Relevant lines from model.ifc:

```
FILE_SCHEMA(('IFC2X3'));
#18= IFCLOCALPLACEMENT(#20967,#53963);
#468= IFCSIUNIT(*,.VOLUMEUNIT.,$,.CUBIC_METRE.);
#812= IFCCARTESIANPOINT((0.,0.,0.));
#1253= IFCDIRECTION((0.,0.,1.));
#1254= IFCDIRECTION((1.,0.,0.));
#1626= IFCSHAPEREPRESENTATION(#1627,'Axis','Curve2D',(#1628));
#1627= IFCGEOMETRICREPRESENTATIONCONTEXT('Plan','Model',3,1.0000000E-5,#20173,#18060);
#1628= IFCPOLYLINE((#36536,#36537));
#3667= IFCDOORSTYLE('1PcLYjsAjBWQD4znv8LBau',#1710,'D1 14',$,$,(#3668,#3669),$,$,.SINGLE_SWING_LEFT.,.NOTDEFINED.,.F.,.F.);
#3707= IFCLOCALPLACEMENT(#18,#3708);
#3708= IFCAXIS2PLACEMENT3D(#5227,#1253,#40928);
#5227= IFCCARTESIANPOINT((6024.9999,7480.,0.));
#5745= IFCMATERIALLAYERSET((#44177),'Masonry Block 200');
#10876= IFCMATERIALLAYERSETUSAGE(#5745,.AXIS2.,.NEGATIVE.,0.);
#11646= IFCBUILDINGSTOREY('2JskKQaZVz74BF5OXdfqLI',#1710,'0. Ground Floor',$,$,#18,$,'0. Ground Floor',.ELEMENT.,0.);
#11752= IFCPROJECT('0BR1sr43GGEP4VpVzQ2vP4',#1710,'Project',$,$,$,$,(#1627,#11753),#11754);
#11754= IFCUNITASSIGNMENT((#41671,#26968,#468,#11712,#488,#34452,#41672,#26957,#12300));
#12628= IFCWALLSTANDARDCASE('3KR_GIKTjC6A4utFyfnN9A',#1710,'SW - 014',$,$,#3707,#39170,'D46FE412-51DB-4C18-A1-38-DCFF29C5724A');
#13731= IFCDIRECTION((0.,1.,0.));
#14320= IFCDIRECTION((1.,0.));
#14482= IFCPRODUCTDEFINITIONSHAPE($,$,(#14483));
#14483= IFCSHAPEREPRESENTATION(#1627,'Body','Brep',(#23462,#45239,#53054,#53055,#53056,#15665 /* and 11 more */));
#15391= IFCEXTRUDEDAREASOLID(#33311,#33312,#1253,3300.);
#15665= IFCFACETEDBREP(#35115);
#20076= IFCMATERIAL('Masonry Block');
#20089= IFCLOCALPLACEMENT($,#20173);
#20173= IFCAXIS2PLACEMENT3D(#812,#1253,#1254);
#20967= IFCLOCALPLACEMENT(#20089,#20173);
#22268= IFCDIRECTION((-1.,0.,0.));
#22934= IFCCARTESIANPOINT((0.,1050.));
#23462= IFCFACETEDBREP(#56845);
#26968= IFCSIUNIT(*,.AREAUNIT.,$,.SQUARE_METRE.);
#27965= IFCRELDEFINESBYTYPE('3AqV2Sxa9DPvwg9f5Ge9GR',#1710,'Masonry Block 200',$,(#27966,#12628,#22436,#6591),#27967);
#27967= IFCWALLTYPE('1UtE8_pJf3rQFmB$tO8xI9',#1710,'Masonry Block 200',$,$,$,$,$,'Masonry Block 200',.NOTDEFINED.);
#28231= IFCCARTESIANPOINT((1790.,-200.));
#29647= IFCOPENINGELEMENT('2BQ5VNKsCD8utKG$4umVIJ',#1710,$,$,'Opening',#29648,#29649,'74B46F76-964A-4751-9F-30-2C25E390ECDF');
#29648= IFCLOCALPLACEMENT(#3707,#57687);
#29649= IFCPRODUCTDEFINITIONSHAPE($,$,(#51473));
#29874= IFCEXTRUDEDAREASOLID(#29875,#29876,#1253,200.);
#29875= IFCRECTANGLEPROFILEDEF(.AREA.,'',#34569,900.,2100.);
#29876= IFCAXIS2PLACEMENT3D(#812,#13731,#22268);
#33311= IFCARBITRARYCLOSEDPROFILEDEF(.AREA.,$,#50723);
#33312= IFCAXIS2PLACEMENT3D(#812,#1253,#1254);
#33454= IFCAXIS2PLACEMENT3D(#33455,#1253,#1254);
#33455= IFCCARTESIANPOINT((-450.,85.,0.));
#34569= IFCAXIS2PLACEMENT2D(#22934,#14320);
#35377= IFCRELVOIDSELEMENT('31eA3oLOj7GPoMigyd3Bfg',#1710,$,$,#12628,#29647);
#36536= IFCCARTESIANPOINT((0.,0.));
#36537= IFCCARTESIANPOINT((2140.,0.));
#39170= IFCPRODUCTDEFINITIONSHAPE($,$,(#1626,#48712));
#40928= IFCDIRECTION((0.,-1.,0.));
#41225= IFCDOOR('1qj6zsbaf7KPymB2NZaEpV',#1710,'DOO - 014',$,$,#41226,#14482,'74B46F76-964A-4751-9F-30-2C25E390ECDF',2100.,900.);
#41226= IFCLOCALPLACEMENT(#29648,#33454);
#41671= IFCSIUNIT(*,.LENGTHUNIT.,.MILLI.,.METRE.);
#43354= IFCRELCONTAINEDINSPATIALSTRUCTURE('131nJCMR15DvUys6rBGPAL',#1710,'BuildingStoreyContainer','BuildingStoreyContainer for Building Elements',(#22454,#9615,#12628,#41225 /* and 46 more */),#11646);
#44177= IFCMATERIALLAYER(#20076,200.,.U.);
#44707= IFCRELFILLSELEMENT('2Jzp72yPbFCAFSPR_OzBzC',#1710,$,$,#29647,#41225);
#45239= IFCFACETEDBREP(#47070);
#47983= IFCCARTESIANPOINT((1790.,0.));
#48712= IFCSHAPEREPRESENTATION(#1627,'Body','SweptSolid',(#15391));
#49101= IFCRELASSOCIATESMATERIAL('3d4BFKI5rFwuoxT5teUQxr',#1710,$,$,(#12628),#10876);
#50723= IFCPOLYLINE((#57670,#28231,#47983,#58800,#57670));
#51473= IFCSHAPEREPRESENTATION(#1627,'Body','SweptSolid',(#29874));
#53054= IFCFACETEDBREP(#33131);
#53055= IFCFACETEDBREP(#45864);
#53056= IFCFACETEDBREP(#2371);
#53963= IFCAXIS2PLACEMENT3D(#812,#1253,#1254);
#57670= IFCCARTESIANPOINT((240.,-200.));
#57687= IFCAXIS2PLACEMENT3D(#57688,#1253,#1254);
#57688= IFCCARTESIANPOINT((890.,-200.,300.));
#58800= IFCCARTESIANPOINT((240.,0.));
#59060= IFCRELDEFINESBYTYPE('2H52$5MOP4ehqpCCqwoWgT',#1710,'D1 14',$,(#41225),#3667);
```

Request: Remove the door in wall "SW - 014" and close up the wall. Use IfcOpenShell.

```python
import ifcopenshell
import ifcopenshell.api.feature
import ifcopenshell.api.root
import ifcopenshell.geom
import ifcopenshell.util.shape

model = ifcopenshell.open("model.ifc")
settings = ifcopenshell.geom.settings()


def volume(element):
    """Net volume in cubic metres, openings subtracted."""
    shape = ifcopenshell.geom.create_shape(settings, element)
    return ifcopenshell.util.shape.get_volume(shape.geometry)


door = model.by_guid("1qj6zsbaf7KPymB2NZaEpV")
opening = door.FillsVoids[0].RelatingOpeningElement
wall = opening.VoidsElements[0].RelatingBuildingElement
before = volume(wall)

ifcopenshell.api.root.remove_product(model, product=door)
ifcopenshell.api.feature.remove_feature(model, feature=opening)

after = volume(wall)

print(f"wall volume {before:.3f} -> {after:.3f} m3")

model.write("model_updated.ifc")
```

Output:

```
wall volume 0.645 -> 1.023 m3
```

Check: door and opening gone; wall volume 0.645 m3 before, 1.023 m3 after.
